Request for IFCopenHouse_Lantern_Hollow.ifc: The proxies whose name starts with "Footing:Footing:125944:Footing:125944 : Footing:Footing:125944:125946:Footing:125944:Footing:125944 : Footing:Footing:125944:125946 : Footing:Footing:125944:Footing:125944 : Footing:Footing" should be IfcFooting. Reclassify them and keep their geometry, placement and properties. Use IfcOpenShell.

First a look at what the model holds.

```python
import re

import ifcopenshell

model = ifcopenshell.open("IFCopenHouse_Lantern_Hollow.ifc")
print(model.schema)
seen = {}
for e in model.by_type("IfcBuildingElementProxy"):
    name = re.sub(r":\d+(:\d+)?$", "", e.Name or "")  # drop the element id that some exporters append
    seen[name] = seen.get(name, 0) + 1
for name, count in sorted(seen.items()):
    print(count, "x", name)
```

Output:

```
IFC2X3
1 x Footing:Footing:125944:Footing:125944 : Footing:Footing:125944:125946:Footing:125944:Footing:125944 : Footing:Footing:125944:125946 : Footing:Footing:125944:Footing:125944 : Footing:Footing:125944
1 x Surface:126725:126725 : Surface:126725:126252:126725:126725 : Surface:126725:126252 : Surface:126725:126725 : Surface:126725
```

```python
import ifcopenshell
import ifcopenshell.api.root

model = ifcopenshell.open("IFCopenHouse_Lantern_Hollow.ifc")

proxies = [e.id() for e in model.by_type("IfcBuildingElementProxy") if (e.Name or "").startswith("Footing:Footing:125944:Footing:125944 : Footing:Footing:125944:125946:Footing:125944:Footing:125944 : Footing:Footing:125944:125946 : Footing:Footing:125944:Footing:125944 : Footing:Footing")]
for step_id in proxies:
    proxy = model.by_id(step_id)
    ifcopenshell.api.root.reassign_class(model, product=proxy, ifc_class="IfcFooting", predefined_type="NOTDEFINED")

print(sum(model.by_id(i).is_a("IfcFooting") for i in proxies), "reclassified")

model.write("IFCopenHouse_Lantern_Hollow_edited.ifc")
```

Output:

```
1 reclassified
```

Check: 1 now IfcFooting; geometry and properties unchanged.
